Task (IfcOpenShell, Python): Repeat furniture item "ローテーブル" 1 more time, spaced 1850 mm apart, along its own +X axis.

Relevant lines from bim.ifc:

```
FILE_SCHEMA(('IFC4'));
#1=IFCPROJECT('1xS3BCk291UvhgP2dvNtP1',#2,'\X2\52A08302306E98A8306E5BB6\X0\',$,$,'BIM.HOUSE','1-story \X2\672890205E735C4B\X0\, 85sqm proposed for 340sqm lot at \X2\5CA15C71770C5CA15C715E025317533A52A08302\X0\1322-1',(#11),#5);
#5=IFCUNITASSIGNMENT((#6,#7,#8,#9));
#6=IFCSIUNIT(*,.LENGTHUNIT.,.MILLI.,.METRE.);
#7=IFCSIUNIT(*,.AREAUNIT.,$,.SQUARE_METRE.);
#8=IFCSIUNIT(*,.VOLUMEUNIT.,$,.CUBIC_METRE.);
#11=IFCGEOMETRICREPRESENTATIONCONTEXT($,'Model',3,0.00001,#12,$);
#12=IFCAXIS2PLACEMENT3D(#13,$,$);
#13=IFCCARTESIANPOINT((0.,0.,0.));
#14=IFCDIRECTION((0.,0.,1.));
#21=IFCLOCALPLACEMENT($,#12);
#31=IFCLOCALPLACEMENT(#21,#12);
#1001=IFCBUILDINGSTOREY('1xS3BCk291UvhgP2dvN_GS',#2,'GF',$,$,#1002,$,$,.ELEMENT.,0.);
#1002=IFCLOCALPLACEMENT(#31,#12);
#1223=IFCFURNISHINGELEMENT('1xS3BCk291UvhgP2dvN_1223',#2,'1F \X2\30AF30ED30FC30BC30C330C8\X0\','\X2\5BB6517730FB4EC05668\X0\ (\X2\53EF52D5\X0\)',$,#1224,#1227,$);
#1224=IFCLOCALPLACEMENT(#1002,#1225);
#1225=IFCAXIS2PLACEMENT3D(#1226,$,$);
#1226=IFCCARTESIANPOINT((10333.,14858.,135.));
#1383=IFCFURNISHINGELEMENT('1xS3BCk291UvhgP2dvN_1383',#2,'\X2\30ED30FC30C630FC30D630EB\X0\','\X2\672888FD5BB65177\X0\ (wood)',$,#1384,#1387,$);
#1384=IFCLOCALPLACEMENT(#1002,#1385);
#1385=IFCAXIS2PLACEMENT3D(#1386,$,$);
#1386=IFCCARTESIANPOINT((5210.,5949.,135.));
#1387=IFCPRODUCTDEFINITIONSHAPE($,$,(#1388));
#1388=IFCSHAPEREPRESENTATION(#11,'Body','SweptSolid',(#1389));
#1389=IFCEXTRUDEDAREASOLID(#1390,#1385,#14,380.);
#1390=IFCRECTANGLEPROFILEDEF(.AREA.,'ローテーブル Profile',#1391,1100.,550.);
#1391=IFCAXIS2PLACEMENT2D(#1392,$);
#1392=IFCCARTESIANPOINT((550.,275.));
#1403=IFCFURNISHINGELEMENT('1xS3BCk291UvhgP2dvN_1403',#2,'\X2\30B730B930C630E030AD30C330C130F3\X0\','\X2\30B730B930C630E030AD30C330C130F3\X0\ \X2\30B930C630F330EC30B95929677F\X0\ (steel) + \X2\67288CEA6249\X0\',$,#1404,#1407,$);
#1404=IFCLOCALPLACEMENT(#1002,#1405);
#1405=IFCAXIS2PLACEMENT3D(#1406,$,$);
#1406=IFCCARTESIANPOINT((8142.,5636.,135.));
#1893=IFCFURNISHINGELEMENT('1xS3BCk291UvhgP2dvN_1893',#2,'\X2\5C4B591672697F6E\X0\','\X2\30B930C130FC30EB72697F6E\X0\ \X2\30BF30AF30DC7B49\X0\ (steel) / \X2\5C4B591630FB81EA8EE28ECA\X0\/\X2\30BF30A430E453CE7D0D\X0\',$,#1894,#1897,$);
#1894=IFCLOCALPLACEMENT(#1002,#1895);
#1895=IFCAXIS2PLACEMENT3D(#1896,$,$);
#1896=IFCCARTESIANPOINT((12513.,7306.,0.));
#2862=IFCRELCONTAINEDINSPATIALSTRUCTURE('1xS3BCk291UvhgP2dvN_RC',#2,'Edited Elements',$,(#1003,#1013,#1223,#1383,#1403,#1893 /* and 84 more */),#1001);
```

```python
import ifcopenshell
import ifcopenshell.api.geometry
import ifcopenshell.api.root
import ifcopenshell.util.element
import ifcopenshell.util.placement

model = ifcopenshell.open("bim.ifc")


def reuse_history(source, copy):
    """copy_class also copies each property set's owner history, people and application; keep the originals."""
    for rel in copy.IsDefinedBy:
        if rel.is_a("IfcRelDefinesByProperties") and (history := rel.RelatingPropertyDefinition.OwnerHistory):
            rel.RelatingPropertyDefinition.OwnerHistory = source.OwnerHistory
            ifcopenshell.util.element.remove_deep2(model, history)


source = model.by_id(1383)
base = ifcopenshell.util.placement.get_local_placement(source.ObjectPlacement)
step = base[:3, 0] * 1850.0

for i in range(1, 2):
    copy = ifcopenshell.api.root.copy_class(model, product=source)
    copy.Representation = ifcopenshell.util.element.copy_deep(
        model, source.Representation, exclude=["IfcGeometricRepresentationContext", "IfcRepresentationMap"]
    )
    reuse_history(source, copy)
    matrix = base.copy()
    matrix[:3, 3] += i * step
    print("added at", matrix[:3, 3].round(3) + 0.0)
    ifcopenshell.api.geometry.edit_object_placement(model, product=copy, matrix=matrix, is_si=False)

model.write("bim_edited.ifc")
```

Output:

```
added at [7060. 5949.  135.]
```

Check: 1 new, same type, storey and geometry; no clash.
